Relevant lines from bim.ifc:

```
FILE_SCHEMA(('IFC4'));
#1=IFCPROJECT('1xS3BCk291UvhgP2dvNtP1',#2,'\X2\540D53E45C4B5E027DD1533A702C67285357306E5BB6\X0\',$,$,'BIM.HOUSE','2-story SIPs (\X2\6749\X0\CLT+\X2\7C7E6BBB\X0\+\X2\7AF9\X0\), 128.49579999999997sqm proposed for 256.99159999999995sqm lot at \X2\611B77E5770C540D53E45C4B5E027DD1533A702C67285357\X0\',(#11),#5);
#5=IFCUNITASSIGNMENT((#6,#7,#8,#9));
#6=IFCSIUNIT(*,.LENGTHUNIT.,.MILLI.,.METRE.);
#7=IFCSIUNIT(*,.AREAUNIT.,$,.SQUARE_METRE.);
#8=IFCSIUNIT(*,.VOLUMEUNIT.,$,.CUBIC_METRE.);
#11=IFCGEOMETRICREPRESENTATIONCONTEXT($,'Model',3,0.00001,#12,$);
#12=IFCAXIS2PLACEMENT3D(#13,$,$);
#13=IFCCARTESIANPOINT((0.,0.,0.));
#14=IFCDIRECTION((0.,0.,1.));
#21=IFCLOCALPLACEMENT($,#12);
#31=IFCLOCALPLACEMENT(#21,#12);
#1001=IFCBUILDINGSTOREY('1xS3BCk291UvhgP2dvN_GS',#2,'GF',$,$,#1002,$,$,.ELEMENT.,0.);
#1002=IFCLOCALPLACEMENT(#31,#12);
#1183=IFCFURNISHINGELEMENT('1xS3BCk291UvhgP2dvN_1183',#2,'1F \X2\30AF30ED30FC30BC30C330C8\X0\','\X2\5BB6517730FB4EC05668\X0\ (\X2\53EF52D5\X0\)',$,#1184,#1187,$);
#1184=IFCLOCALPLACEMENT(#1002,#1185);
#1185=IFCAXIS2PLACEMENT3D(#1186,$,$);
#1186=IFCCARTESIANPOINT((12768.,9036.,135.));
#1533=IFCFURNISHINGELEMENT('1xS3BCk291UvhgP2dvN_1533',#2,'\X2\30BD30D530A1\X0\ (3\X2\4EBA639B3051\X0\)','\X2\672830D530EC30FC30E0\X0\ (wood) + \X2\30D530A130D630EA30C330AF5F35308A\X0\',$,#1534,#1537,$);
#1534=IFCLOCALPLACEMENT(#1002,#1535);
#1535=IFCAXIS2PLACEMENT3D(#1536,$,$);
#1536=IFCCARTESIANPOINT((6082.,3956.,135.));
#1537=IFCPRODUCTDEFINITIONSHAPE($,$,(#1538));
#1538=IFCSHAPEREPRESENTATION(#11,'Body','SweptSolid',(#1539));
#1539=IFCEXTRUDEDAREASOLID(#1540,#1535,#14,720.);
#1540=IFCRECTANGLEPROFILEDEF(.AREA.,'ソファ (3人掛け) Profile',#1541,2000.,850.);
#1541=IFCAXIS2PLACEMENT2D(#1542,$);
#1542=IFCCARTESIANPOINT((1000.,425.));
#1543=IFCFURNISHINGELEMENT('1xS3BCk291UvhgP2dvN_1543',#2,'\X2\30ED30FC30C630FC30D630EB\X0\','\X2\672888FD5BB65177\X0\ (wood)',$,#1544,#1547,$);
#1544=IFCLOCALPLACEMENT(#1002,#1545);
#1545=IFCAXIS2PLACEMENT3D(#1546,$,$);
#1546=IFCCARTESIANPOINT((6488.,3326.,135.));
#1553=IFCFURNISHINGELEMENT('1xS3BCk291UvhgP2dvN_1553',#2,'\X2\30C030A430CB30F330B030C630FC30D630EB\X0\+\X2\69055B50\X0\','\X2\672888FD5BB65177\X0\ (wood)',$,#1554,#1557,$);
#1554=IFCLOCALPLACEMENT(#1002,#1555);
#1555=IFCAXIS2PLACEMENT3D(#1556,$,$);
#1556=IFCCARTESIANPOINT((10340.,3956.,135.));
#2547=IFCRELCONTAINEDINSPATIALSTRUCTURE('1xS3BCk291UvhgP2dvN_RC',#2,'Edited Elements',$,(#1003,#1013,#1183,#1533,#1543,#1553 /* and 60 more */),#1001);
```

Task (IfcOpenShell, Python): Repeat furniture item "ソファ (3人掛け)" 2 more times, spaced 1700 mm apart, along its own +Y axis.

```python
import ifcopenshell
import ifcopenshell.api.geometry
import ifcopenshell.api.root
import ifcopenshell.util.element
import ifcopenshell.util.placement

model = ifcopenshell.open("bim.ifc")


def reuse_history(source, copy):
    """copy_class also copies each property set's owner history, people and application; keep the originals."""
    for rel in copy.IsDefinedBy:
        if rel.is_a("IfcRelDefinesByProperties") and (history := rel.RelatingPropertyDefinition.OwnerHistory):
            rel.RelatingPropertyDefinition.OwnerHistory = source.OwnerHistory
            ifcopenshell.util.element.remove_deep2(model, history)


source = model.by_id(1533)
base = ifcopenshell.util.placement.get_local_placement(source.ObjectPlacement)
step = base[:3, 1] * 1700.0

for i in range(1, 3):
    copy = ifcopenshell.api.root.copy_class(model, product=source)
    copy.Representation = ifcopenshell.util.element.copy_deep(
        model, source.Representation, exclude=["IfcGeometricRepresentationContext", "IfcRepresentationMap"]
    )
    reuse_history(source, copy)
    matrix = base.copy()
    matrix[:3, 3] += i * step
    print("added at", matrix[:3, 3].round(3) + 0.0)
    ifcopenshell.api.geometry.edit_object_placement(model, product=copy, matrix=matrix, is_si=False)

model.write("bim_rev.ifc")
```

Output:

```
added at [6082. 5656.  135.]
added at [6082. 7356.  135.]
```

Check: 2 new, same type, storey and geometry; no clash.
